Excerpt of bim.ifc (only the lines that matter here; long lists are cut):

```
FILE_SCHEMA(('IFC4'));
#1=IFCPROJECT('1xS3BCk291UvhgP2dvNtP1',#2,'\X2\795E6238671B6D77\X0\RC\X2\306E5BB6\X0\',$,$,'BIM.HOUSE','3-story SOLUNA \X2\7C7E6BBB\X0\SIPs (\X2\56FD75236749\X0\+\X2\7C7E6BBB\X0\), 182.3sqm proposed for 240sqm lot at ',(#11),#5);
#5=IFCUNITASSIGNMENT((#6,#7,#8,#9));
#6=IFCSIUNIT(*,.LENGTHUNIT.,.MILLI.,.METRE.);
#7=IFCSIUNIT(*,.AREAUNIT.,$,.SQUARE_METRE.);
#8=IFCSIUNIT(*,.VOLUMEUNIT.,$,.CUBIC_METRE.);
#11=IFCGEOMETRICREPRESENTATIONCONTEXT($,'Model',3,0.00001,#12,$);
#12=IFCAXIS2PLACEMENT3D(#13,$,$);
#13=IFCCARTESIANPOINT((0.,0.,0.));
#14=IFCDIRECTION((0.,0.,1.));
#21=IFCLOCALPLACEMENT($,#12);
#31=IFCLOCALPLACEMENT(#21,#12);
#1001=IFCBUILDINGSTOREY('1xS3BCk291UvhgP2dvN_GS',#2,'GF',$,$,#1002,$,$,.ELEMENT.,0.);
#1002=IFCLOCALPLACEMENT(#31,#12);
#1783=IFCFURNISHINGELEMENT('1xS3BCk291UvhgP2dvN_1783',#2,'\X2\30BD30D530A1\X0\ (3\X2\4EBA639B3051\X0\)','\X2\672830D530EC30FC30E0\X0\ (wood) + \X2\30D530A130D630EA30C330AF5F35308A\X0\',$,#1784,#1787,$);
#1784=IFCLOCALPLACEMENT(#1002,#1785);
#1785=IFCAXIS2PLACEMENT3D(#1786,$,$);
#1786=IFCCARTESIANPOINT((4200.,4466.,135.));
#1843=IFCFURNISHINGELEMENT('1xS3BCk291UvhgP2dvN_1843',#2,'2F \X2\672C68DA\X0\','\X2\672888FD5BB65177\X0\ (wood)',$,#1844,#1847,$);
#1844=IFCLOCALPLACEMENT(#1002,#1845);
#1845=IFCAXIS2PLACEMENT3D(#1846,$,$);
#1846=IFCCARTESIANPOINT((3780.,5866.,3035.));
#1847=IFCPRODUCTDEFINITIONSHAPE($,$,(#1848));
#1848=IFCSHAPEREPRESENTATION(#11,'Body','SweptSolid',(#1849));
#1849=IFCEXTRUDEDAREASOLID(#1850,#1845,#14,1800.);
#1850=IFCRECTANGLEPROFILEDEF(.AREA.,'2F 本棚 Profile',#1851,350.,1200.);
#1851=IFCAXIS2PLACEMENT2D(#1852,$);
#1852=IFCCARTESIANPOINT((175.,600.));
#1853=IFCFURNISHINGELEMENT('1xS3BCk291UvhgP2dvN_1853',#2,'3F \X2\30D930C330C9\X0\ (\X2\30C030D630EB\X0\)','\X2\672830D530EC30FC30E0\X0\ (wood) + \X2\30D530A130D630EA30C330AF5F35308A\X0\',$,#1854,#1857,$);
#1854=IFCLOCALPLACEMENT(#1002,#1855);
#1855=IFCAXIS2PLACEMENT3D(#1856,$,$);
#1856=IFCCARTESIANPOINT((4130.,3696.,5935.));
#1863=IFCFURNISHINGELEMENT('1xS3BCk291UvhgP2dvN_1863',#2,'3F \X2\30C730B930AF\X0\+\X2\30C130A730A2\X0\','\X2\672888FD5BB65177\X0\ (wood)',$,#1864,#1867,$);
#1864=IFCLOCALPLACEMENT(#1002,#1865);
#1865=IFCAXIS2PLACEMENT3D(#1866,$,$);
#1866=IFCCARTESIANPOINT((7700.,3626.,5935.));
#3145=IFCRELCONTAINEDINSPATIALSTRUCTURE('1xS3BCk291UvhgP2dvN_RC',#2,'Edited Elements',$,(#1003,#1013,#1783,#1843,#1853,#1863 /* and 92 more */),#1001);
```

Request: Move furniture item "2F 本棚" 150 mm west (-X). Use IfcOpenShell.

```python
import ifcopenshell
import ifcopenshell.api.geometry
import ifcopenshell.util.placement

model = ifcopenshell.open("bim.ifc")

item = model.by_guid("1xS3BCk291UvhgP2dvN_1843")
matrix = ifcopenshell.util.placement.get_local_placement(item.ObjectPlacement)
matrix[0, 3] -= 150.0
ifcopenshell.api.geometry.edit_object_placement(model, product=item, matrix=matrix, is_si=False)

print(ifcopenshell.util.placement.get_local_placement(item.ObjectPlacement).round(3) + 0.0)

model.write("bim-out.ifc")
```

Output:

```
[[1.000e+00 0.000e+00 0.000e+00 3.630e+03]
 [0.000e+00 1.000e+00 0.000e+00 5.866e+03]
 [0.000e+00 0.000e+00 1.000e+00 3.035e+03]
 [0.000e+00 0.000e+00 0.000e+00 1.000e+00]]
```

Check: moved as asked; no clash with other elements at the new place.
